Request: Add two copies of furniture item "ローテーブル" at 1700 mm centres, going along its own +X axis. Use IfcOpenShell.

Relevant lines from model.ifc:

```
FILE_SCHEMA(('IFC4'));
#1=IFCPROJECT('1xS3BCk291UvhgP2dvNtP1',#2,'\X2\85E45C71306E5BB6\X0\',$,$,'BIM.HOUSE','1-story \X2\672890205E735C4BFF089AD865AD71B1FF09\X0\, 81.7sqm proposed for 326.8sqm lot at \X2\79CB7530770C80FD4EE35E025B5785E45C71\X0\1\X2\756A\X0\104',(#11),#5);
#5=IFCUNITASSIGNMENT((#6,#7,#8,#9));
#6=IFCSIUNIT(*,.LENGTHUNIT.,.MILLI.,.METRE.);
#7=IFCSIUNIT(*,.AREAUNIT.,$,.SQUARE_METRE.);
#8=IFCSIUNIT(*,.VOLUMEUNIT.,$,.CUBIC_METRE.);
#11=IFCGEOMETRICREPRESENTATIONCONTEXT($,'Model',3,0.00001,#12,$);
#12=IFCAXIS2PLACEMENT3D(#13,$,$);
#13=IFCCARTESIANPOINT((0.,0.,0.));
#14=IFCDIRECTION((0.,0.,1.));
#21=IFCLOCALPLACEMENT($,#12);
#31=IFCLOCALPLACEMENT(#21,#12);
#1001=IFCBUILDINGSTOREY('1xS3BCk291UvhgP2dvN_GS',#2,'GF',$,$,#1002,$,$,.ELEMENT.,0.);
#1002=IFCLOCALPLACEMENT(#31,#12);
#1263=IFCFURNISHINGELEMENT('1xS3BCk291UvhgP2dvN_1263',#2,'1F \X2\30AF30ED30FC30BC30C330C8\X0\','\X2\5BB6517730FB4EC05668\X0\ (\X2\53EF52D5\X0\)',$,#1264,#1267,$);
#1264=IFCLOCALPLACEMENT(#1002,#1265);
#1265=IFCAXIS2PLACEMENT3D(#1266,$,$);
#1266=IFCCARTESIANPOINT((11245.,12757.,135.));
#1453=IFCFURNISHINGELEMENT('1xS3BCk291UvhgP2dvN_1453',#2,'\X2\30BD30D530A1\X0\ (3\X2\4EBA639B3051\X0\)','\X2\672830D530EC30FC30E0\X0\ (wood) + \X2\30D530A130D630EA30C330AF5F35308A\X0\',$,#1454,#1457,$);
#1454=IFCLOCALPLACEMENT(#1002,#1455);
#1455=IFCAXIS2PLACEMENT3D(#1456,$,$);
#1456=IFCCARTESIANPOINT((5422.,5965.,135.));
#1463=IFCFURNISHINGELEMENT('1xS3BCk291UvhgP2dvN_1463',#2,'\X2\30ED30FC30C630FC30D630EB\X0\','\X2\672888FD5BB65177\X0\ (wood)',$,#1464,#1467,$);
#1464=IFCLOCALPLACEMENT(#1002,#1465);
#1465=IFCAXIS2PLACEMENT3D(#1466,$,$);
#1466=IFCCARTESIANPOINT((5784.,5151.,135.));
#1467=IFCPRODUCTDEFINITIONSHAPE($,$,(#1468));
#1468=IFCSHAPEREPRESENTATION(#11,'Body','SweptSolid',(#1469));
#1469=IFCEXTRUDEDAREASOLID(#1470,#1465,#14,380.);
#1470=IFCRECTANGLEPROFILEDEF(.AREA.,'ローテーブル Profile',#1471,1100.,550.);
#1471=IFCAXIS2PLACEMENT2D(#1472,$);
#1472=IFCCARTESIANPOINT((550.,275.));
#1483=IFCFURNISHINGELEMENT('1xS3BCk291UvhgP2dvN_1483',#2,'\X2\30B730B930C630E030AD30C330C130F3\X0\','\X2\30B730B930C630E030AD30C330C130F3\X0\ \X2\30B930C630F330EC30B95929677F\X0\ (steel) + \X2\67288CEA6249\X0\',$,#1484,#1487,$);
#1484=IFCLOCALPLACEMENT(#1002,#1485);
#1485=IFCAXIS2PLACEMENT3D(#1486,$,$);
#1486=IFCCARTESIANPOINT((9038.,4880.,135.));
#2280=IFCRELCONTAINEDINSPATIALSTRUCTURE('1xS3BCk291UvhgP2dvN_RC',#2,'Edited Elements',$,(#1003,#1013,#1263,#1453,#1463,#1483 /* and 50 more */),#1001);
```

```python
import ifcopenshell
import ifcopenshell.api.geometry
import ifcopenshell.api.root
import ifcopenshell.util.element
import ifcopenshell.util.placement

model = ifcopenshell.open("model.ifc")


def reuse_history(source, copy):
    """copy_class also copies each property set's owner history, people and application; keep the originals."""
    for rel in copy.IsDefinedBy:
        if rel.is_a("IfcRelDefinesByProperties") and (history := rel.RelatingPropertyDefinition.OwnerHistory):
            rel.RelatingPropertyDefinition.OwnerHistory = source.OwnerHistory
            ifcopenshell.util.element.remove_deep2(model, history)


source = model.by_id(1463)
base = ifcopenshell.util.placement.get_local_placement(source.ObjectPlacement)
step = base[:3, 0] * 1700.0

for i in range(1, 3):
    copy = ifcopenshell.api.root.copy_class(model, product=source)
    copy.Representation = ifcopenshell.util.element.copy_deep(
        model, source.Representation, exclude=["IfcGeometricRepresentationContext", "IfcRepresentationMap"]
    )
    reuse_history(source, copy)
    matrix = base.copy()
    matrix[:3, 3] += i * step
    print("added at", matrix[:3, 3].round(3) + 0.0)
    ifcopenshell.api.geometry.edit_object_placement(model, product=copy, matrix=matrix, is_si=False)

model.write("model_edited.ifc")
```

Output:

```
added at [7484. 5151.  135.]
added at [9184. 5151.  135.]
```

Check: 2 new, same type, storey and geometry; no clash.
